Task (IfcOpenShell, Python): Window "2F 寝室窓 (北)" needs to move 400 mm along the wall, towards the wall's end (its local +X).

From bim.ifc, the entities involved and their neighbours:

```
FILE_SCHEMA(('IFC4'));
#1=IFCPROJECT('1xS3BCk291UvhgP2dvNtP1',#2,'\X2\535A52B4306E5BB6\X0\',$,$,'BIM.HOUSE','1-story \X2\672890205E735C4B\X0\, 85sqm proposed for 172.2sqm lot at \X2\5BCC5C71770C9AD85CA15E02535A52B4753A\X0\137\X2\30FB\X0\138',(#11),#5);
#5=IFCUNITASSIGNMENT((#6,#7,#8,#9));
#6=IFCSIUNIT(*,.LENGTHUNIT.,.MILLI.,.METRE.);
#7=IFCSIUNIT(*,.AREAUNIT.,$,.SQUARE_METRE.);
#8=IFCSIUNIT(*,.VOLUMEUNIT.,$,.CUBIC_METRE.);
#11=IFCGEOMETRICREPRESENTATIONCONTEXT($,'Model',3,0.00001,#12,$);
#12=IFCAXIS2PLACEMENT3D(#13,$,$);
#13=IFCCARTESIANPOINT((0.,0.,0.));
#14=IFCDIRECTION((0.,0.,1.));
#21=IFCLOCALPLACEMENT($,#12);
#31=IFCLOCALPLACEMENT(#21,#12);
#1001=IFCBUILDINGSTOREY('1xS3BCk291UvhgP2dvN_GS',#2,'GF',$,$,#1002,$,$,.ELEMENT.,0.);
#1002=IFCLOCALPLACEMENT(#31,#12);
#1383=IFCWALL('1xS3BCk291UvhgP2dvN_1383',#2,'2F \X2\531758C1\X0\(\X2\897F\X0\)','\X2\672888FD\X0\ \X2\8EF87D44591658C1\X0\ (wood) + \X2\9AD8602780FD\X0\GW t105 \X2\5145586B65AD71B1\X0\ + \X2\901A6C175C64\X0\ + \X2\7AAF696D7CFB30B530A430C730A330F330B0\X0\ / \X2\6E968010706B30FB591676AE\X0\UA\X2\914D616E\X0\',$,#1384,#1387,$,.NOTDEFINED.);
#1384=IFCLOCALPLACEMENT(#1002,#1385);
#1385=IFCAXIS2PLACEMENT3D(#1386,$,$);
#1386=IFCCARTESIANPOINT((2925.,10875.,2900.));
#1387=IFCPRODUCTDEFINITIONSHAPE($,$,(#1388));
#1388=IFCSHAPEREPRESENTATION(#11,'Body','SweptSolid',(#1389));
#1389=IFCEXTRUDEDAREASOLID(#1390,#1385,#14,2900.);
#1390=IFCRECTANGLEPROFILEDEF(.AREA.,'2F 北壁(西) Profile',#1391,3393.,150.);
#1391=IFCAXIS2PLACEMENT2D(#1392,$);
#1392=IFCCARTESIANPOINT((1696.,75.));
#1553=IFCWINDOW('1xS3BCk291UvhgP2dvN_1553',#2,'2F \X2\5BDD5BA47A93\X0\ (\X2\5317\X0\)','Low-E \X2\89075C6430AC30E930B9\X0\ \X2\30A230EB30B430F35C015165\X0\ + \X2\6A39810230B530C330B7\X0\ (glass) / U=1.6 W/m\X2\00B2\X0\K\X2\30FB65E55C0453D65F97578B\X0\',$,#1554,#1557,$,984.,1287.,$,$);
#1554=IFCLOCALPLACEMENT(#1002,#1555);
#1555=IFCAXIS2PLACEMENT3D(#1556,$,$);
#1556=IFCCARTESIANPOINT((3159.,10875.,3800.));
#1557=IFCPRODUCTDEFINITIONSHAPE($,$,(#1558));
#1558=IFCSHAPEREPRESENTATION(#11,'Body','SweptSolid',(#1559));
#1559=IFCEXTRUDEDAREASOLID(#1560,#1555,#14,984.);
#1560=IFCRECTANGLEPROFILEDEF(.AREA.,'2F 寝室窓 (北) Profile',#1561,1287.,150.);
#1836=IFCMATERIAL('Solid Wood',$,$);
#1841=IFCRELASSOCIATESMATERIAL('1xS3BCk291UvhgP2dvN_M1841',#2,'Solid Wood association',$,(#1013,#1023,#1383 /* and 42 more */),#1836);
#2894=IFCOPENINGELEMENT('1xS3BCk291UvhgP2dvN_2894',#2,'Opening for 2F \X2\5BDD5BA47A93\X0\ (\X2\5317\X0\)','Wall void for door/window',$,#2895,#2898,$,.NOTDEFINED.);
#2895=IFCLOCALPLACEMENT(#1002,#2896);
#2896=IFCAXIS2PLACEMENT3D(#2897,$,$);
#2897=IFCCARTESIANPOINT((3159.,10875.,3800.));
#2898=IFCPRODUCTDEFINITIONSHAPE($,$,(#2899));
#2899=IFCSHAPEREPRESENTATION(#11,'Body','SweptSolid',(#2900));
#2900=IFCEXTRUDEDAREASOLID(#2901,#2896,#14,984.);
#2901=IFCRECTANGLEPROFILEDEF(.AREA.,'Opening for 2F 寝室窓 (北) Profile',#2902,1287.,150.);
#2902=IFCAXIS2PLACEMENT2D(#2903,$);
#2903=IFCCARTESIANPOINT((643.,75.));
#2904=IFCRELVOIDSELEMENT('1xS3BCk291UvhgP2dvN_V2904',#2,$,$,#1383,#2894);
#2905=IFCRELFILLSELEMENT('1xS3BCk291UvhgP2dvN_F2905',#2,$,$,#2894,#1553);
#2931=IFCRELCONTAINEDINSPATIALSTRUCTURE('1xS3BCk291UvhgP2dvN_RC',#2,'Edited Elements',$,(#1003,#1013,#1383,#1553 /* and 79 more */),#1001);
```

```python
import ifcopenshell
import ifcopenshell.api.geometry
import ifcopenshell.util.placement
import ifcopenshell.util.unit

model = ifcopenshell.open("bim.ifc")
unit_scale = ifcopenshell.util.unit.calculate_unit_scale(model)

window = model.by_id(1553)
opening = window.FillsVoids[0].RelatingOpeningElement
wall = opening.VoidsElements[0].RelatingBuildingElement

wall_matrix = ifcopenshell.util.placement.get_local_placement(wall.ObjectPlacement)
shift = wall_matrix[:3, 0] * 0.4 / unit_scale
before = ifcopenshell.util.placement.get_local_placement(window.ObjectPlacement)[:3, 3].copy()

# The window is not placed relative to its opening, so move both.
for product in (opening, window):
    matrix = ifcopenshell.util.placement.get_local_placement(product.ObjectPlacement)
    matrix[:3, 3] += shift
    ifcopenshell.api.geometry.edit_object_placement(model, product=product, matrix=matrix, is_si=False)

after = ifcopenshell.util.placement.get_local_placement(window.ObjectPlacement)[:3, 3]
print("window moved by", (after - before).round(3) + 0.0)

model.write("bim_v2.ifc")
```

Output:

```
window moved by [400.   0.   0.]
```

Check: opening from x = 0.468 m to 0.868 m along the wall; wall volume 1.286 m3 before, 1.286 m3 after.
